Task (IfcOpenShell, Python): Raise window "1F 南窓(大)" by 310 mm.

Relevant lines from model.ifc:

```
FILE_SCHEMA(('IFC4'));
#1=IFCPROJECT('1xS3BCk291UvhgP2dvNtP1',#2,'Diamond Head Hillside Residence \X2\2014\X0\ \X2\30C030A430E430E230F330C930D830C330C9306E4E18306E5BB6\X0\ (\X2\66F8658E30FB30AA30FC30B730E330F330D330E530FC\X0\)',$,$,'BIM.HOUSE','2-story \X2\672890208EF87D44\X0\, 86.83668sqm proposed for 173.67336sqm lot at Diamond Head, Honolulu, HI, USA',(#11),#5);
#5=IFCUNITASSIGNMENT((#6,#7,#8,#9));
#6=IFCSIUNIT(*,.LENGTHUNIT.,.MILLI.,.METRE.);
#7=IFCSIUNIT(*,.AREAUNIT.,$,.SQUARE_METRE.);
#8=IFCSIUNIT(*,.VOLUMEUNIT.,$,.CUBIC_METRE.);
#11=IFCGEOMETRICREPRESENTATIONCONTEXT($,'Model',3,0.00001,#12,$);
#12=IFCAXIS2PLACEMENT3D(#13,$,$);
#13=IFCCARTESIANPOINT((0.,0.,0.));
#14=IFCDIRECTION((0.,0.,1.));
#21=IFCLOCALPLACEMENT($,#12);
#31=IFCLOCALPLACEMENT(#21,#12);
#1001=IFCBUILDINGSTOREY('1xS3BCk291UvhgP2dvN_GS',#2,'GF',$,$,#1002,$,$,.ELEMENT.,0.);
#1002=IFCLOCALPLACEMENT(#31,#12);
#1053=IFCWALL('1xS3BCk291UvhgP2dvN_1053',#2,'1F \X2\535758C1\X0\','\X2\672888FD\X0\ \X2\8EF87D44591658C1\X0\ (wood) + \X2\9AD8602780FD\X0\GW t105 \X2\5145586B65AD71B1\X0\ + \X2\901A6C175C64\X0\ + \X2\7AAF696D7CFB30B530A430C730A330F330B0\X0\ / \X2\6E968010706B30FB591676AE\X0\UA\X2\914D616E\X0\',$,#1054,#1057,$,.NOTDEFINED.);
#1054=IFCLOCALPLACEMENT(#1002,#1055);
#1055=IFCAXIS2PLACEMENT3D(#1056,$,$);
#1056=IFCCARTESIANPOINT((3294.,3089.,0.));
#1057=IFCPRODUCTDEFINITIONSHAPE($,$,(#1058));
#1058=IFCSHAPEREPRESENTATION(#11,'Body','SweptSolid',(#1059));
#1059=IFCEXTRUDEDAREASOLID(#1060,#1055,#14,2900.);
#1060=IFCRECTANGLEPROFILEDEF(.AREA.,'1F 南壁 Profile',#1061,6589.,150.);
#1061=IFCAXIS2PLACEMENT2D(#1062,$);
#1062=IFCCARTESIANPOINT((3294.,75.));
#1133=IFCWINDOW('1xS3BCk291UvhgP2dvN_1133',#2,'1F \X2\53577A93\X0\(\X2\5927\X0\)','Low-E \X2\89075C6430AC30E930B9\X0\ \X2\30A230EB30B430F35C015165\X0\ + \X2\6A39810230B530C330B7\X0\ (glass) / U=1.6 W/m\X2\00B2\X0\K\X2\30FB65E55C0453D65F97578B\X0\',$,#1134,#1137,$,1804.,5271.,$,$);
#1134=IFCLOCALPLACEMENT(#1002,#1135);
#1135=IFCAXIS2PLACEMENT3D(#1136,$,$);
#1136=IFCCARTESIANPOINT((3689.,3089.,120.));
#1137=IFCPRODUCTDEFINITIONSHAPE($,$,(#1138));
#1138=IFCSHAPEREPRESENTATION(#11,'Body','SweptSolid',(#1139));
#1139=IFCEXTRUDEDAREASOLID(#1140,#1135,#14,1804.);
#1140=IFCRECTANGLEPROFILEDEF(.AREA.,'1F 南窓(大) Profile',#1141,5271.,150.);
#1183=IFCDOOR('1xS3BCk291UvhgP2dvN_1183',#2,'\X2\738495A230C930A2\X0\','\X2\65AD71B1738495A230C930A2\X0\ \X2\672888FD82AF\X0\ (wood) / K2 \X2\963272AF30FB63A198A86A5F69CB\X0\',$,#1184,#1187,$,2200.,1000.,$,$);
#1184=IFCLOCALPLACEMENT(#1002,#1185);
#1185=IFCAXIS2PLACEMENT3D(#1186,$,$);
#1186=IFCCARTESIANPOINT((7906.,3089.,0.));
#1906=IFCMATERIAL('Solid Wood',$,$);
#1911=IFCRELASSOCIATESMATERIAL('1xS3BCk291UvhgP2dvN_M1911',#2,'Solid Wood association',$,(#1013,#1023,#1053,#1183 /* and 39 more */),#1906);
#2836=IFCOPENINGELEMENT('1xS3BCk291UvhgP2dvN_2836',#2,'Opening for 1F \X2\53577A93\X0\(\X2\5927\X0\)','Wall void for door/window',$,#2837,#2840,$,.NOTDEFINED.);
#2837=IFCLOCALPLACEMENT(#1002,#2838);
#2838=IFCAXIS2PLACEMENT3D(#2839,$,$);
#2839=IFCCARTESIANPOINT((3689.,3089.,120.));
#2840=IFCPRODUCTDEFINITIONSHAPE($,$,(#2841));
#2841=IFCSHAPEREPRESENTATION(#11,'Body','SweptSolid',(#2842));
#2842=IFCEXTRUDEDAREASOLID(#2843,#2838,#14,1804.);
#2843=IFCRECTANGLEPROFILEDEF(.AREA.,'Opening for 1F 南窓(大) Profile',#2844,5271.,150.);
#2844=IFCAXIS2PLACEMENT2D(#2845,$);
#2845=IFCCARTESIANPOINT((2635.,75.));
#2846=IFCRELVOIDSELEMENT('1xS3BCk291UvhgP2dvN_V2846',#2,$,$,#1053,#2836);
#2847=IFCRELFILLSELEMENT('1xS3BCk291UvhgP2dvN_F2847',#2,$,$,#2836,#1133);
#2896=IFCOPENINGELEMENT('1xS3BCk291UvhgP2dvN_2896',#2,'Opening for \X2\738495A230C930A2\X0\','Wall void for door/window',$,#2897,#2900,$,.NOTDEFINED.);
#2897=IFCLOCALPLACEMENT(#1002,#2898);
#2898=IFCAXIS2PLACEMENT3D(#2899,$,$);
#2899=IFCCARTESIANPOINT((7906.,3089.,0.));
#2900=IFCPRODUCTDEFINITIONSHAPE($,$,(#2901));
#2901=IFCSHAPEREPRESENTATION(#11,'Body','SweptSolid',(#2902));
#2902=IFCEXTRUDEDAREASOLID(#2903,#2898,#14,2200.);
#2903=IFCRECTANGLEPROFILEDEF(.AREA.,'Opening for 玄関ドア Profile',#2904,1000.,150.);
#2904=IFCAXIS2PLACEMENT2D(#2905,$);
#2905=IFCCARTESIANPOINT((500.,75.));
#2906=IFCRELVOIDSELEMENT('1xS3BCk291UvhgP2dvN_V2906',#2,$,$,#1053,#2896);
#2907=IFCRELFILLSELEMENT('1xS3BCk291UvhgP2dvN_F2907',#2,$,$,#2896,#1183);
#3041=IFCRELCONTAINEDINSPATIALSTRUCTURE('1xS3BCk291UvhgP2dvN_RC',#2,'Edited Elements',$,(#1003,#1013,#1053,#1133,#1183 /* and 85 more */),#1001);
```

```python
import numpy as np
import ifcopenshell
import ifcopenshell.api.geometry
import ifcopenshell.util.placement
import ifcopenshell.util.unit

model = ifcopenshell.open("model.ifc")
unit_scale = ifcopenshell.util.unit.calculate_unit_scale(model)

window = model.by_id(1133)
opening = window.FillsVoids[0].RelatingOpeningElement
dz = 310.0

shift = np.array([0.0, 0.0, dz])
# The window is not placed relative to its opening, so move both.
for product in (opening, window):
    matrix = ifcopenshell.util.placement.get_local_placement(product.ObjectPlacement)
    matrix[:3, 3] += shift
    ifcopenshell.api.geometry.edit_object_placement(model, product=product, matrix=matrix, is_si=False)

print(f"moved by {dz * unit_scale:+.3f} m")

model.write("model_rev.ifc")
```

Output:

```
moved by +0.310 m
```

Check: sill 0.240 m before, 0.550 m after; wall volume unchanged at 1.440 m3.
